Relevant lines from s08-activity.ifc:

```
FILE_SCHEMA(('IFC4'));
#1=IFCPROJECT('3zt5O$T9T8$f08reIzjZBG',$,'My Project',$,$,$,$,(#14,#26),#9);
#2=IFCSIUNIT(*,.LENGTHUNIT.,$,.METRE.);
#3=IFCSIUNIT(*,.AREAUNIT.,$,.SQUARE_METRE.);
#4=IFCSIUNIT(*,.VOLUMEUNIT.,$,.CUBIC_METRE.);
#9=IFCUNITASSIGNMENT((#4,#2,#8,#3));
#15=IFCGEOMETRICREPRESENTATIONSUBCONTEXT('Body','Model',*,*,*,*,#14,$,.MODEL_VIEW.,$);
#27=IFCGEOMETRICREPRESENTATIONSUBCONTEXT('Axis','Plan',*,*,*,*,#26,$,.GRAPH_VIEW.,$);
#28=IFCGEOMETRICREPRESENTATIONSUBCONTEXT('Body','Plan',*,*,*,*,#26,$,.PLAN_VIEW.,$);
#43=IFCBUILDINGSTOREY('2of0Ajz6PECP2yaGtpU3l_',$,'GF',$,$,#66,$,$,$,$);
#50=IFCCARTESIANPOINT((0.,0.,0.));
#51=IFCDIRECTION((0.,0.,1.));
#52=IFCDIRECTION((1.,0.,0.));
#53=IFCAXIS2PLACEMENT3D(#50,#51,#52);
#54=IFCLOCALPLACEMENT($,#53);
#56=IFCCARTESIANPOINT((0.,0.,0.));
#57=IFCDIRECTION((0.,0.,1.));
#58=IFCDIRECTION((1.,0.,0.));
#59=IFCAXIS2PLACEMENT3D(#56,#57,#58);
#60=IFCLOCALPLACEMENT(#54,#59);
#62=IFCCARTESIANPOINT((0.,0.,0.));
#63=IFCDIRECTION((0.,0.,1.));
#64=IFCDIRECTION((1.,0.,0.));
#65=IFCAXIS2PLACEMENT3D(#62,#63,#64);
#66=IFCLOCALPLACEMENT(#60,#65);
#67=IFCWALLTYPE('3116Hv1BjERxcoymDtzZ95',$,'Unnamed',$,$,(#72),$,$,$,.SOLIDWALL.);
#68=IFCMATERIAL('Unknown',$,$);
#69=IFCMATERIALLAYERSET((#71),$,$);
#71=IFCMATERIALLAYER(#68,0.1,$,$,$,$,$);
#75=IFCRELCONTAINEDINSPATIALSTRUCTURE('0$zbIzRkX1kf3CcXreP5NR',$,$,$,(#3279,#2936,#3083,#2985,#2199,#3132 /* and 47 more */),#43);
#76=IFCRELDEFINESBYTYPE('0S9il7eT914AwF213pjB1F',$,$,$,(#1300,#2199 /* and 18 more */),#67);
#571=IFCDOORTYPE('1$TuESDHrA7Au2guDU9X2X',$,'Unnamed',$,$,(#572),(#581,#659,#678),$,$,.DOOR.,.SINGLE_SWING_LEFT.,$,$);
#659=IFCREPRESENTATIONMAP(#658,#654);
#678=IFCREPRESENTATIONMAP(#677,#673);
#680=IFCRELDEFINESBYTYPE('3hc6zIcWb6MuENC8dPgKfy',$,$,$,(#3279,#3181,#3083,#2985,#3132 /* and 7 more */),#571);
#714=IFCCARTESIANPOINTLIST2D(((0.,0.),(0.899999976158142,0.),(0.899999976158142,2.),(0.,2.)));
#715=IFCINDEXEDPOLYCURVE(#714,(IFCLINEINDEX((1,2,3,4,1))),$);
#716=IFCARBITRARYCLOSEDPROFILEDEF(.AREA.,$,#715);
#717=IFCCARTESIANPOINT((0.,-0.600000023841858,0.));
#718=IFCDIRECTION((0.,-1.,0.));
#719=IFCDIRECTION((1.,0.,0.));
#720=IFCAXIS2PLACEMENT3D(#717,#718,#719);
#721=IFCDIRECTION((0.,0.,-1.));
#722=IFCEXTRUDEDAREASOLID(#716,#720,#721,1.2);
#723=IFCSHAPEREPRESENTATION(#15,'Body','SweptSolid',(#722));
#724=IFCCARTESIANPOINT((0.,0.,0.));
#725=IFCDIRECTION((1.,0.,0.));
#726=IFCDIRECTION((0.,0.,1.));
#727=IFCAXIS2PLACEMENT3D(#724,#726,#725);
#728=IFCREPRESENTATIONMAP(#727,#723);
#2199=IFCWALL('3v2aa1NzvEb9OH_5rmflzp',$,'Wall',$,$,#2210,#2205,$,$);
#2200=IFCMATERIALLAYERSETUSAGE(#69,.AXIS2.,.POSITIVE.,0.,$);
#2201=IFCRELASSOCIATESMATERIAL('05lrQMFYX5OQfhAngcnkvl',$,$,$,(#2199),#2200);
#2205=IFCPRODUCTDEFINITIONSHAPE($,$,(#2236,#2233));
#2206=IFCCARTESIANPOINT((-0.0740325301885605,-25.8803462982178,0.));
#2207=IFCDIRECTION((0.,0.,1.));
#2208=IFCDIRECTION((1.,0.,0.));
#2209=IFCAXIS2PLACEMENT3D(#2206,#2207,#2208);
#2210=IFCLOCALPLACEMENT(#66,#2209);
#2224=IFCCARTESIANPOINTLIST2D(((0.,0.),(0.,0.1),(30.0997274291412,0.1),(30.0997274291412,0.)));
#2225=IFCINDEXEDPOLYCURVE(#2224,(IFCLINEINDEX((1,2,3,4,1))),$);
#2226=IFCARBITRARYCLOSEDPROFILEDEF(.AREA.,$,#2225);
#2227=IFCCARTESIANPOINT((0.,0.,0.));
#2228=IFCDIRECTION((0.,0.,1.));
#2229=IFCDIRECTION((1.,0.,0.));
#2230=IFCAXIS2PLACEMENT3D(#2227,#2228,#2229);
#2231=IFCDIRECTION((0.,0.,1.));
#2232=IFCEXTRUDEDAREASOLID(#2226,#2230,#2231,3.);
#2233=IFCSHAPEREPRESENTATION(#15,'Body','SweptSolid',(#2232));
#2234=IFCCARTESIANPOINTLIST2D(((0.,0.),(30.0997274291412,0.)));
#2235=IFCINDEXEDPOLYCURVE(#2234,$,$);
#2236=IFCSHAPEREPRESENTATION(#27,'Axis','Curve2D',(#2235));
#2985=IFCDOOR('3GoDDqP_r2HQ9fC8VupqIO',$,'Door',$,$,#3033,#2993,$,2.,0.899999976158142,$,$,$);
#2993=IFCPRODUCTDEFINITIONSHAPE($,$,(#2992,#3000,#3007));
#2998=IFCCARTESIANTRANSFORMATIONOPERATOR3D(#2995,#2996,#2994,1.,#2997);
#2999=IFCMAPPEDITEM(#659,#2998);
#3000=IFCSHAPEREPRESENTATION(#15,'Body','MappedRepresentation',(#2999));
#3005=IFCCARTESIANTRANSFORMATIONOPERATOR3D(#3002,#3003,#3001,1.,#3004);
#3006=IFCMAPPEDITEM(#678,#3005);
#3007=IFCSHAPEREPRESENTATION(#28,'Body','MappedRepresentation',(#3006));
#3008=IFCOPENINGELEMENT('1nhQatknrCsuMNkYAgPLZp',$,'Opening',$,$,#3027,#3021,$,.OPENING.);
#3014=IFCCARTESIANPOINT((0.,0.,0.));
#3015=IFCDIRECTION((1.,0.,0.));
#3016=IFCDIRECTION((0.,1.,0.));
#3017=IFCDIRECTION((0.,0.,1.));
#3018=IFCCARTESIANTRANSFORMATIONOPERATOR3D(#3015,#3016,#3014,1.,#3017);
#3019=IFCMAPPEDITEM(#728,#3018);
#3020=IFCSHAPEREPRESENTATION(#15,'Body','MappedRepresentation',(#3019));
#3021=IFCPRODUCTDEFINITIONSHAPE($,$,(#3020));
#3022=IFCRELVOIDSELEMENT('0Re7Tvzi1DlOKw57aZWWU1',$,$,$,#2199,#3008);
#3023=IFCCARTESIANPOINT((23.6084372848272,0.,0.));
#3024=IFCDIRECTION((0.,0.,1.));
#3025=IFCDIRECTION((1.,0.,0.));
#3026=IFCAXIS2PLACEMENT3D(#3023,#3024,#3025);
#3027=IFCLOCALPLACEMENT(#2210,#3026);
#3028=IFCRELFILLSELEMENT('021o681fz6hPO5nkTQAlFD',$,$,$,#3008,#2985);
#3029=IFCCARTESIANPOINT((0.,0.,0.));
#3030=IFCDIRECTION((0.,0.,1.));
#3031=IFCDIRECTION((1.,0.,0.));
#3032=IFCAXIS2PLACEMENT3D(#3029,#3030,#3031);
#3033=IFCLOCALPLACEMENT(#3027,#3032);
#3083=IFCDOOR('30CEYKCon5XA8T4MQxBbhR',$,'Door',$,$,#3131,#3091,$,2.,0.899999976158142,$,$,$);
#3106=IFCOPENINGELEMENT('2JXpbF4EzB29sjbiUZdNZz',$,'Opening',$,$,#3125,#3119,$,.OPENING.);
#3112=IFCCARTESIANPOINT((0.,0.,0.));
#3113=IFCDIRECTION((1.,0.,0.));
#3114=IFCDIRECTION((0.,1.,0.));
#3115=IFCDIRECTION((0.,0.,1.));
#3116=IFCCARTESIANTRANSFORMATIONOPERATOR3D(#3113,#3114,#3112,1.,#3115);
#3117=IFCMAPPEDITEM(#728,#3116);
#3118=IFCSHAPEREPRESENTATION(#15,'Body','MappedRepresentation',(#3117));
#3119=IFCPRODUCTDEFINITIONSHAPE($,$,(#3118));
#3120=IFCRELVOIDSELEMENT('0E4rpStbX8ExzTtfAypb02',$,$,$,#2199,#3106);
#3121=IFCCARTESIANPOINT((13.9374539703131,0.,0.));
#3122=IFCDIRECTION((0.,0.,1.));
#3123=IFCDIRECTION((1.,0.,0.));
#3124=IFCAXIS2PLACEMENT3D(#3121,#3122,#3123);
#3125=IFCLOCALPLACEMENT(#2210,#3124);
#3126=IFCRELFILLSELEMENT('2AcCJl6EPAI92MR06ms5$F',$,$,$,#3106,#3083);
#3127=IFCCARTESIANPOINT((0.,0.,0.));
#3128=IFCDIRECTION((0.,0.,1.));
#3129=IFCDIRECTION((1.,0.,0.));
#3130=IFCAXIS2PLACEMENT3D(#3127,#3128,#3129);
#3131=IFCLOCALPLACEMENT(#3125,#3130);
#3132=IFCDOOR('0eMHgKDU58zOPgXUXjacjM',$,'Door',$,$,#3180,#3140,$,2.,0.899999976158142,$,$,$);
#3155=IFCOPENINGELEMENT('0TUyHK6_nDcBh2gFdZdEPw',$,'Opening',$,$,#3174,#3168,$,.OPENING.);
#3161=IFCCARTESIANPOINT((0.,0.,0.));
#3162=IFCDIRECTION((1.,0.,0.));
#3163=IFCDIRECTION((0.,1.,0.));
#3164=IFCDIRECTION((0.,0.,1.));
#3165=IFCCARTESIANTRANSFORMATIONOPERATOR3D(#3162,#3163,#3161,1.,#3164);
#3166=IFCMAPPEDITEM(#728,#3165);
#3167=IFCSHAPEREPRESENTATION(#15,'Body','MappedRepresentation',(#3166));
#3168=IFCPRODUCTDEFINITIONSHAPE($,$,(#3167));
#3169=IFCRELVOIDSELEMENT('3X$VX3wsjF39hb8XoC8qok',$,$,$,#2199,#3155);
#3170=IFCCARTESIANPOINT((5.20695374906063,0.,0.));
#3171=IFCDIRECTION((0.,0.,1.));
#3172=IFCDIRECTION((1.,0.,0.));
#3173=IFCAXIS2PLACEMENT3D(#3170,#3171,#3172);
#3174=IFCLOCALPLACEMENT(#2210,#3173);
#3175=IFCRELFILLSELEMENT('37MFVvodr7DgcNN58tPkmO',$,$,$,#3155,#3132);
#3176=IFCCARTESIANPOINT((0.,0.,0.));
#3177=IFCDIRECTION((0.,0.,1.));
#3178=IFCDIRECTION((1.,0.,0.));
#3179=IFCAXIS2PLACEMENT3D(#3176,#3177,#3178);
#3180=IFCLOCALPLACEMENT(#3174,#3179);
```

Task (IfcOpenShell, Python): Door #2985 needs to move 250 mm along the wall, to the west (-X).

```python
import ifcopenshell
import ifcopenshell.api.geometry
import ifcopenshell.util.placement

model = ifcopenshell.open("s08-activity.ifc")

door = model.by_guid("3GoDDqP_r2HQ9fC8VupqIO")
opening = door.FillsVoids[0].RelatingOpeningElement
wall = opening.VoidsElements[0].RelatingBuildingElement

wall_matrix = ifcopenshell.util.placement.get_local_placement(wall.ObjectPlacement)
shift = wall_matrix[:3, 0] * -0.25
before = ifcopenshell.util.placement.get_local_placement(door.ObjectPlacement)[:3, 3].copy()

# The door is placed relative to its opening, so it follows when the opening moves.
matrix = ifcopenshell.util.placement.get_local_placement(opening.ObjectPlacement)
matrix[:3, 3] += shift
ifcopenshell.api.geometry.edit_object_placement(
    model, product=opening, matrix=matrix, is_si=False, should_transform_children=True
)

after = ifcopenshell.util.placement.get_local_placement(door.ObjectPlacement)[:3, 3]
print("door moved by", (after - before).round(3) + 0.0)

model.write("s08-activity-out.ifc")
```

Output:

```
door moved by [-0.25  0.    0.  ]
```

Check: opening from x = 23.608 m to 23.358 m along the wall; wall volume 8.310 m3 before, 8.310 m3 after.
